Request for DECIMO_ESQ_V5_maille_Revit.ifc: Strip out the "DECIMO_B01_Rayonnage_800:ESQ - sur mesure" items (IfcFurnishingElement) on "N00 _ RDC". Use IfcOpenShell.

First a look at what the model holds.

```python
import ifcopenshell
import ifcopenshell.util.element

model = ifcopenshell.open("DECIMO_ESQ_V5_maille_Revit.ifc")
print(model.schema)
storey = next(s for s in model.by_type("IfcBuildingStorey") if s.Name == "N00 _ RDC")
furniture = [e for e in ifcopenshell.util.element.get_decomposition(storey) if e.is_a("IfcFurnishingElement")]
seen = {}
for e in furniture:
    element_type = ifcopenshell.util.element.get_type(e)
    name = element_type.Name if element_type not in (None, e) else None
    seen[name] = seen.get(name, 0) + 1
for name, count in sorted(seen.items(), key=str):
    print(count, "x", name)
```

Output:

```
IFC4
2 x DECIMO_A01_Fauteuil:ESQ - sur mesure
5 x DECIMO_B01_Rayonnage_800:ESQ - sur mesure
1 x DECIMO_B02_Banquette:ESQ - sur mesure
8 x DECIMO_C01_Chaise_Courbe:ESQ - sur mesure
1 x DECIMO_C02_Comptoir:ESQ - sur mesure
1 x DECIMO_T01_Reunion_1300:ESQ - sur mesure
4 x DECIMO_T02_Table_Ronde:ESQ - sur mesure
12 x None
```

```python
import ifcopenshell
import ifcopenshell.api.root
import ifcopenshell.util.element

model = ifcopenshell.open("DECIMO_ESQ_V5_maille_Revit.ifc")

storey = next(s for s in model.by_type("IfcBuildingStorey") if s.Name == "N00 _ RDC")
furniture = [e for e in ifcopenshell.util.element.get_decomposition(storey) if e.is_a("IfcFurnishingElement")]
targets = [e for e in furniture if (t := ifcopenshell.util.element.get_type(e)) not in (None, e) and t.Name == "DECIMO_B01_Rayonnage_800:ESQ - sur mesure"]

for e in targets:
    ifcopenshell.api.root.remove_product(model, product=e)
print(len(targets), "removed")

model.write("DECIMO_ESQ_V5_maille_Revit_updated.ifc")
```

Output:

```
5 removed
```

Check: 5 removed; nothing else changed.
